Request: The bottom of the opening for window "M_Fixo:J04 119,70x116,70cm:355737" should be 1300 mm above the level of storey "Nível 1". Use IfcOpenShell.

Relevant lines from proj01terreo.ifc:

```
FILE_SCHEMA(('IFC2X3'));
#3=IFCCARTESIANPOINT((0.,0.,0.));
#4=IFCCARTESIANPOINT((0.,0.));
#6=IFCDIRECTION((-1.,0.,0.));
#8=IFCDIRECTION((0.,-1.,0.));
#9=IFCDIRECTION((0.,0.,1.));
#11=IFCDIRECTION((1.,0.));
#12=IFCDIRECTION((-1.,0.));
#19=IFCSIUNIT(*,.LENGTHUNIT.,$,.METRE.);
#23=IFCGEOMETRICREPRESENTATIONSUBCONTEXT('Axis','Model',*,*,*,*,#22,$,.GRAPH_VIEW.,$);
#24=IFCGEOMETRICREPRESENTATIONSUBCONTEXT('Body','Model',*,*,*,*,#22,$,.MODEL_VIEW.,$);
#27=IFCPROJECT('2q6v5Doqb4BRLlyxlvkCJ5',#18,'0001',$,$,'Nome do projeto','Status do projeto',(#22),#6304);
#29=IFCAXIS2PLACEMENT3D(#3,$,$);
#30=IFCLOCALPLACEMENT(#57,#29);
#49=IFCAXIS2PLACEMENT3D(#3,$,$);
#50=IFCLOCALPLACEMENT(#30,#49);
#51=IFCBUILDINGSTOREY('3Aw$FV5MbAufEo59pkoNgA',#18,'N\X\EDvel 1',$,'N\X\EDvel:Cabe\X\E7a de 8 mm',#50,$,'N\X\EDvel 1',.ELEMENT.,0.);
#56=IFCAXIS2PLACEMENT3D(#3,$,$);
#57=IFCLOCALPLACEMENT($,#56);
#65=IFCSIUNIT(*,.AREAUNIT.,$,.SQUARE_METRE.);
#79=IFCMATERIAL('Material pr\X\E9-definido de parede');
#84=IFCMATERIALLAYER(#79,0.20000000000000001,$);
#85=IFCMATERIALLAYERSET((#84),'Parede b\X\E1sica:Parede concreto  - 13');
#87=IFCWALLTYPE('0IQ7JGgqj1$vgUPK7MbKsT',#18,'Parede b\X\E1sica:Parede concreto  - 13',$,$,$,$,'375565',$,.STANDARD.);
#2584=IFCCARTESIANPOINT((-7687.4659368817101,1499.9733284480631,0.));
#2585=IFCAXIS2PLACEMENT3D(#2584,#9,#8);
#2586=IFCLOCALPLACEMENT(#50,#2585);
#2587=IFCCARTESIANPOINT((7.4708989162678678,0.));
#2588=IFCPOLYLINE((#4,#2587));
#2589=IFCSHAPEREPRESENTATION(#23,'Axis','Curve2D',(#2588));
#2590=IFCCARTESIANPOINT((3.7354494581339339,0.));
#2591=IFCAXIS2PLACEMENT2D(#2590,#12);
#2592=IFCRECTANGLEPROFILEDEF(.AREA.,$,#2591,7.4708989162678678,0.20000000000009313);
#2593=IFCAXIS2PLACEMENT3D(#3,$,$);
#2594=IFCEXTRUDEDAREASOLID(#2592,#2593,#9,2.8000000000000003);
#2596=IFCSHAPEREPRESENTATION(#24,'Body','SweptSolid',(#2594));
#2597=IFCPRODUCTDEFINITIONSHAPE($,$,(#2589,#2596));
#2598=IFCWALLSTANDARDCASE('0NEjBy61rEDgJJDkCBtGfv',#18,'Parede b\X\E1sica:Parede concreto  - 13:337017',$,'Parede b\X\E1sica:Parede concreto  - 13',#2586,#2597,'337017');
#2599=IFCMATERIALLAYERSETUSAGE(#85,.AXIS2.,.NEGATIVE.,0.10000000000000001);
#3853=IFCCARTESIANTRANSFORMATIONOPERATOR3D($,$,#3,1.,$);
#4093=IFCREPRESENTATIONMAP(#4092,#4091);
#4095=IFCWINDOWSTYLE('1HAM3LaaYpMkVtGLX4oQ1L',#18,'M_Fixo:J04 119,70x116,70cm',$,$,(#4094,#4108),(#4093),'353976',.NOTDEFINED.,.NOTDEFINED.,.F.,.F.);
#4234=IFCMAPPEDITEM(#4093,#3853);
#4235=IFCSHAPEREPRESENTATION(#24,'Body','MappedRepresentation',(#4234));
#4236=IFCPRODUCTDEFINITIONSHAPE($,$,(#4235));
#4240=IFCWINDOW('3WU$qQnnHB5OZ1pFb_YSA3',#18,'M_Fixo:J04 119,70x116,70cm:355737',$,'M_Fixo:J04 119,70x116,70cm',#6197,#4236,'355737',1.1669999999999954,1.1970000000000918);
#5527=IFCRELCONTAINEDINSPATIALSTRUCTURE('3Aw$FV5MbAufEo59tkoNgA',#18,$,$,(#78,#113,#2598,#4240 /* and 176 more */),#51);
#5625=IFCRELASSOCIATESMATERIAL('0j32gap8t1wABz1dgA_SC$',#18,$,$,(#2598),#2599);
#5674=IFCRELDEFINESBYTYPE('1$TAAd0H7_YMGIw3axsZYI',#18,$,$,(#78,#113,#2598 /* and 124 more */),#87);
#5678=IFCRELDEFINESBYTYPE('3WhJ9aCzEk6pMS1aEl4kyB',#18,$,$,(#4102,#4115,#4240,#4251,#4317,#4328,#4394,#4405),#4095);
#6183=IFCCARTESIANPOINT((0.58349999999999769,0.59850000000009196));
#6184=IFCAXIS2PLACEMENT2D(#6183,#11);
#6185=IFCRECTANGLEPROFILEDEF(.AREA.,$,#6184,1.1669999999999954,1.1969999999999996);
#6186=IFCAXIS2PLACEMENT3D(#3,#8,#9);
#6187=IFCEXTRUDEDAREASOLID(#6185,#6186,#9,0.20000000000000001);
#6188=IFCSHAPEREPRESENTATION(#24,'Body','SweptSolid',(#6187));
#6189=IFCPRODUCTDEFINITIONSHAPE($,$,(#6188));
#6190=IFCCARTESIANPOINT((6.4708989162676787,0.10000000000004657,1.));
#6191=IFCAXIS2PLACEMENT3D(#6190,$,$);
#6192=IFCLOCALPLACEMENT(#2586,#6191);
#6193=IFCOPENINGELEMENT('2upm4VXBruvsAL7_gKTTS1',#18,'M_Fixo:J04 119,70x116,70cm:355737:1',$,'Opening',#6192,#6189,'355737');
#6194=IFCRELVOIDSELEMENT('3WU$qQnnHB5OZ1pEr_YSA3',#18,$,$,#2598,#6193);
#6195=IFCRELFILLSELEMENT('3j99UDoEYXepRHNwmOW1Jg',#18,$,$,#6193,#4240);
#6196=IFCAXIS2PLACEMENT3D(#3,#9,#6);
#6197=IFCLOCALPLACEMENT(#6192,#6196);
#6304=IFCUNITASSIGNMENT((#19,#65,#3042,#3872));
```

```python
import numpy as np
import ifcopenshell
import ifcopenshell.api.geometry
import ifcopenshell.geom
import ifcopenshell.util.element
import ifcopenshell.util.placement
import ifcopenshell.util.shape
import ifcopenshell.util.unit

model = ifcopenshell.open("proj01terreo.ifc")
unit_scale = ifcopenshell.util.unit.calculate_unit_scale(model)

window = model.by_id(4240)
opening = window.FillsVoids[0].RelatingOpeningElement
storey = ifcopenshell.util.element.get_container(window, ifc_class="IfcBuildingStorey")
level = ifcopenshell.util.placement.get_local_placement(storey.ObjectPlacement)[2, 3]

# The opening's origin need not be at the sill, so measure its lowest point.
shape = ifcopenshell.geom.create_shape(ifcopenshell.geom.settings(), opening)
bottom = ifcopenshell.util.shape.get_shape_bottom_elevation(shape, shape.geometry) / unit_scale
dz = level + 1.3 / unit_scale - bottom

shift = np.array([0.0, 0.0, dz])
# The window is placed relative to its opening, so it follows when the opening moves.
matrix = ifcopenshell.util.placement.get_local_placement(opening.ObjectPlacement)
matrix[:3, 3] += shift
ifcopenshell.api.geometry.edit_object_placement(
    model, product=opening, matrix=matrix, is_si=False, should_transform_children=True
)

print(f"moved by {dz * unit_scale:+.3f} m")

model.write("proj01terreo_v2.ifc")
```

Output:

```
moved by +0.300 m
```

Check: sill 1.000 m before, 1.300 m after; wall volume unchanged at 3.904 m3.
